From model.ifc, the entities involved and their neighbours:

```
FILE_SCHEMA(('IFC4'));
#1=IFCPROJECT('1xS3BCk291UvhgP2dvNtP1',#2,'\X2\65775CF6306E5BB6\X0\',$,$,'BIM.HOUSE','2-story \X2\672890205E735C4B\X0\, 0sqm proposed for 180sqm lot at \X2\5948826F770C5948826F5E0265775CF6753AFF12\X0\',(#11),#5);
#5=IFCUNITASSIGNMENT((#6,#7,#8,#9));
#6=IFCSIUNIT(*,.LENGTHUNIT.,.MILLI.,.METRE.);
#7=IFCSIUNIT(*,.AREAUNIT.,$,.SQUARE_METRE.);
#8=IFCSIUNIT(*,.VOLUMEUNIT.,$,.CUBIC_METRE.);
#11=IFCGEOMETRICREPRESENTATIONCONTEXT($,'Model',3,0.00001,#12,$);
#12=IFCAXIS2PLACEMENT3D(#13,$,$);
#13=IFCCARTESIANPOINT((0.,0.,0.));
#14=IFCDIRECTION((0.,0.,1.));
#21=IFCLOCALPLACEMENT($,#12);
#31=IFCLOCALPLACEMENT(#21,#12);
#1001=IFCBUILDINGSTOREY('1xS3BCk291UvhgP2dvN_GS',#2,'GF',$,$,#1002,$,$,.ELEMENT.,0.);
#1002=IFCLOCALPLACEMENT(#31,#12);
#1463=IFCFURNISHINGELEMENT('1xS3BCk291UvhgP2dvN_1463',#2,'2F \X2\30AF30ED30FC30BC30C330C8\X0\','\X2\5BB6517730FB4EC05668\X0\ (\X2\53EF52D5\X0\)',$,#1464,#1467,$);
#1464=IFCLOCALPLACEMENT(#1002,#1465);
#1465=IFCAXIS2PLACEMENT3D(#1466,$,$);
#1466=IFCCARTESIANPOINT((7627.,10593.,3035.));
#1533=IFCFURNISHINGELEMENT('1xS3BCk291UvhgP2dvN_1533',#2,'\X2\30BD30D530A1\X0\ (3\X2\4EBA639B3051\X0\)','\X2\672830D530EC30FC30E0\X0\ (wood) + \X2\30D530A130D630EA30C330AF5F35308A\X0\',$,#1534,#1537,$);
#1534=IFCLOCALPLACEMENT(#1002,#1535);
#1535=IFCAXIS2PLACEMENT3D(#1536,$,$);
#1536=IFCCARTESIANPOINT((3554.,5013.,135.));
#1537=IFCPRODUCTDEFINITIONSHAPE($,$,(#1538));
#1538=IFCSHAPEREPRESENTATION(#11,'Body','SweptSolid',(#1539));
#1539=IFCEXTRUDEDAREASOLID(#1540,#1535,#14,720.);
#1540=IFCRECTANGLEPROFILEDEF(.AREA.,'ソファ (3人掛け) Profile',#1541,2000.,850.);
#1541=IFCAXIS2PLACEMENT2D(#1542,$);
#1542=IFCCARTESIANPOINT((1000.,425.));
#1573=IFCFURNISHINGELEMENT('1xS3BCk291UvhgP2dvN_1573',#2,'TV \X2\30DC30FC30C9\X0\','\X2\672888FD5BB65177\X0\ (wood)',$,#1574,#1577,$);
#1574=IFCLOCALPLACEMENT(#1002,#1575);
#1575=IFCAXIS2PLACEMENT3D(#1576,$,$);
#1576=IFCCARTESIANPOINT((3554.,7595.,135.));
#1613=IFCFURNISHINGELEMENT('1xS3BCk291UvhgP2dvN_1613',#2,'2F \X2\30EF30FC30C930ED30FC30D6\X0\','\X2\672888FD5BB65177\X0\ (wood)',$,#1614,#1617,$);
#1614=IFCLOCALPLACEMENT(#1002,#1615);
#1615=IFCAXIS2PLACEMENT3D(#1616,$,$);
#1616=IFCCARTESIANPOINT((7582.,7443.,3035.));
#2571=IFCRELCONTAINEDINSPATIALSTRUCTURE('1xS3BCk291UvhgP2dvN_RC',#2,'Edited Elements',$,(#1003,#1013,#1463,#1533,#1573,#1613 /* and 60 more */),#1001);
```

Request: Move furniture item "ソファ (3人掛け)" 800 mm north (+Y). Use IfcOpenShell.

```python
import ifcopenshell
import ifcopenshell.api.geometry
import ifcopenshell.util.placement

model = ifcopenshell.open("model.ifc")

item = model.by_guid("1xS3BCk291UvhgP2dvN_1533")
matrix = ifcopenshell.util.placement.get_local_placement(item.ObjectPlacement)
matrix[1, 3] += 800.0
ifcopenshell.api.geometry.edit_object_placement(model, product=item, matrix=matrix, is_si=False)

print(ifcopenshell.util.placement.get_local_placement(item.ObjectPlacement).round(3) + 0.0)

model.write("model_rev.ifc")
```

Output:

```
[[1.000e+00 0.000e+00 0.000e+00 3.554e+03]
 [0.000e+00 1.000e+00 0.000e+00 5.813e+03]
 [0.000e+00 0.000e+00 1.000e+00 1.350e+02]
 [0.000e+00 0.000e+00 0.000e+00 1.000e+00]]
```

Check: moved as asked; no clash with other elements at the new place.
